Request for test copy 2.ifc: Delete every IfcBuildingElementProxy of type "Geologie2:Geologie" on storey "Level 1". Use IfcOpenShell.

First a look at what the model holds.

```python
import ifcopenshell
import ifcopenshell.util.element

model = ifcopenshell.open("test copy 2.ifc")
print(model.schema)
storey = next(s for s in model.by_type("IfcBuildingStorey") if s.Name == "Level 1")
proxies = [e for e in ifcopenshell.util.element.get_decomposition(storey) if e.is_a("IfcBuildingElementProxy")]
seen = {}
for e in proxies:
    element_type = ifcopenshell.util.element.get_type(e)
    name = element_type.Name if element_type not in (None, e) else None
    seen[name] = seen.get(name, 0) + 1
for name, count in sorted(seen.items(), key=str):
    print(count, "x", name)
```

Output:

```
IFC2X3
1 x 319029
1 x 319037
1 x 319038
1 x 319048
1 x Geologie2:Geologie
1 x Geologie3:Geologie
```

```python
import ifcopenshell
import ifcopenshell.api.root
import ifcopenshell.util.element

model = ifcopenshell.open("test copy 2.ifc")

storey = next(s for s in model.by_type("IfcBuildingStorey") if s.Name == "Level 1")
proxies = [e for e in ifcopenshell.util.element.get_decomposition(storey) if e.is_a("IfcBuildingElementProxy")]
targets = [e for e in proxies if (t := ifcopenshell.util.element.get_type(e)) not in (None, e) and t.Name == "Geologie2:Geologie"]

for e in targets:
    ifcopenshell.api.root.remove_product(model, product=e)
print(len(targets), "removed")

model.write("test copy 2_updated.ifc")
```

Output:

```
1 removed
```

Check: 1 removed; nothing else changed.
